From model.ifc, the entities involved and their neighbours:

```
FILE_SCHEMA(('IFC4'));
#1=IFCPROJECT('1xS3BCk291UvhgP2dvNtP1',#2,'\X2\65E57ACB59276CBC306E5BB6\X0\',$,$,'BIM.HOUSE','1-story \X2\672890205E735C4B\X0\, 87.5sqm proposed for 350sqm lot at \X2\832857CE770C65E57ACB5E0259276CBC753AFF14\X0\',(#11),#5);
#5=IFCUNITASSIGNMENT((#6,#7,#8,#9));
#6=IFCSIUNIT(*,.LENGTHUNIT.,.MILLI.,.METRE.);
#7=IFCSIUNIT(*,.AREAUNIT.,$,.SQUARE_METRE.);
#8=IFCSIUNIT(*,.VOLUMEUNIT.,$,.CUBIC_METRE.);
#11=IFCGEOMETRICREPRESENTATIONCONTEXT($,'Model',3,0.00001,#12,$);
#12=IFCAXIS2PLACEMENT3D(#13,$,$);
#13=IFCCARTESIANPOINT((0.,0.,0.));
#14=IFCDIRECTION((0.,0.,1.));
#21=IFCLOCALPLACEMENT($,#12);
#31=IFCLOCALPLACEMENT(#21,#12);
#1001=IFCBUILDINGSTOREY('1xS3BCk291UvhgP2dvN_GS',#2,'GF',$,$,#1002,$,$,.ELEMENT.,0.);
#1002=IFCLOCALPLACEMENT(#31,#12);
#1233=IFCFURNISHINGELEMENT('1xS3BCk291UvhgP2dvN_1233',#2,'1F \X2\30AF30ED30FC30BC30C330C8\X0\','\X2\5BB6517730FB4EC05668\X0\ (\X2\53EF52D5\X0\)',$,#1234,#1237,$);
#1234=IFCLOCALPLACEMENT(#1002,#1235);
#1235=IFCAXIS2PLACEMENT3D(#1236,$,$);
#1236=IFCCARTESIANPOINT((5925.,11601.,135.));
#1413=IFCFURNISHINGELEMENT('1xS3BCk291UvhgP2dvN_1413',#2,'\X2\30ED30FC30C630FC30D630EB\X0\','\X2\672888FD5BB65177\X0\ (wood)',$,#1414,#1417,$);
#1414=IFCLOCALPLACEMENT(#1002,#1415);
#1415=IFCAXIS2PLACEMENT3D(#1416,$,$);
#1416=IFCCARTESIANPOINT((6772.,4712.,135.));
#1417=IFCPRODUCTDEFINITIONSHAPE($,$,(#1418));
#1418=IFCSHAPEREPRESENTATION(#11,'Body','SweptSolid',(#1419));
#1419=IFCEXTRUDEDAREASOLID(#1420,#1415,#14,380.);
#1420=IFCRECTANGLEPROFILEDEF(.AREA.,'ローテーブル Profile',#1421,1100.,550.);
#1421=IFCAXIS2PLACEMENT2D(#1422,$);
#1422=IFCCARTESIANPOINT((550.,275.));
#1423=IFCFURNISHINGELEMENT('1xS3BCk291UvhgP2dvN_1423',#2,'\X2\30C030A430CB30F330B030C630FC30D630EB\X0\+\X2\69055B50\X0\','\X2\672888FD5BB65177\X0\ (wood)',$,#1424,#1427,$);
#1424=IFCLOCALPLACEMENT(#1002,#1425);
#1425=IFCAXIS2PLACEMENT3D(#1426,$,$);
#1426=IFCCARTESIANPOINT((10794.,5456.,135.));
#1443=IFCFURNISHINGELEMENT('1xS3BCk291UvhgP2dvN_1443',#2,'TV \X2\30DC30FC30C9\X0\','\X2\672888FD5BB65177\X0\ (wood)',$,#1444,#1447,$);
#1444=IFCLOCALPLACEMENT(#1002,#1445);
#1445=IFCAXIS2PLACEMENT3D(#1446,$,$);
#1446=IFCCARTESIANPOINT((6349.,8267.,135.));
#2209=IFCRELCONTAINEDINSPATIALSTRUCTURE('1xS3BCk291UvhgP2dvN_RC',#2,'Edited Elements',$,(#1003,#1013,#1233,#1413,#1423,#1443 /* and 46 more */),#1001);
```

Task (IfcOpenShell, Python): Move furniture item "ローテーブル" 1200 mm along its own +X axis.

```python
import ifcopenshell
import ifcopenshell.api.geometry
import ifcopenshell.util.placement

model = ifcopenshell.open("model.ifc")

item = model.by_id(1413)
matrix = ifcopenshell.util.placement.get_local_placement(item.ObjectPlacement)
matrix[:3, 3] += matrix[:3, 0] * 1200.0
ifcopenshell.api.geometry.edit_object_placement(model, product=item, matrix=matrix, is_si=False)

print(ifcopenshell.util.placement.get_local_placement(item.ObjectPlacement).round(3) + 0.0)

model.write("model_v2.ifc")
```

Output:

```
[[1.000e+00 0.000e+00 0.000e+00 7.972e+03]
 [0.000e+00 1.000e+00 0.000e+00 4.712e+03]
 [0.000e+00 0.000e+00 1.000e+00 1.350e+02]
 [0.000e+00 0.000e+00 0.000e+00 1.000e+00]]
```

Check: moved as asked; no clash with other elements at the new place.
